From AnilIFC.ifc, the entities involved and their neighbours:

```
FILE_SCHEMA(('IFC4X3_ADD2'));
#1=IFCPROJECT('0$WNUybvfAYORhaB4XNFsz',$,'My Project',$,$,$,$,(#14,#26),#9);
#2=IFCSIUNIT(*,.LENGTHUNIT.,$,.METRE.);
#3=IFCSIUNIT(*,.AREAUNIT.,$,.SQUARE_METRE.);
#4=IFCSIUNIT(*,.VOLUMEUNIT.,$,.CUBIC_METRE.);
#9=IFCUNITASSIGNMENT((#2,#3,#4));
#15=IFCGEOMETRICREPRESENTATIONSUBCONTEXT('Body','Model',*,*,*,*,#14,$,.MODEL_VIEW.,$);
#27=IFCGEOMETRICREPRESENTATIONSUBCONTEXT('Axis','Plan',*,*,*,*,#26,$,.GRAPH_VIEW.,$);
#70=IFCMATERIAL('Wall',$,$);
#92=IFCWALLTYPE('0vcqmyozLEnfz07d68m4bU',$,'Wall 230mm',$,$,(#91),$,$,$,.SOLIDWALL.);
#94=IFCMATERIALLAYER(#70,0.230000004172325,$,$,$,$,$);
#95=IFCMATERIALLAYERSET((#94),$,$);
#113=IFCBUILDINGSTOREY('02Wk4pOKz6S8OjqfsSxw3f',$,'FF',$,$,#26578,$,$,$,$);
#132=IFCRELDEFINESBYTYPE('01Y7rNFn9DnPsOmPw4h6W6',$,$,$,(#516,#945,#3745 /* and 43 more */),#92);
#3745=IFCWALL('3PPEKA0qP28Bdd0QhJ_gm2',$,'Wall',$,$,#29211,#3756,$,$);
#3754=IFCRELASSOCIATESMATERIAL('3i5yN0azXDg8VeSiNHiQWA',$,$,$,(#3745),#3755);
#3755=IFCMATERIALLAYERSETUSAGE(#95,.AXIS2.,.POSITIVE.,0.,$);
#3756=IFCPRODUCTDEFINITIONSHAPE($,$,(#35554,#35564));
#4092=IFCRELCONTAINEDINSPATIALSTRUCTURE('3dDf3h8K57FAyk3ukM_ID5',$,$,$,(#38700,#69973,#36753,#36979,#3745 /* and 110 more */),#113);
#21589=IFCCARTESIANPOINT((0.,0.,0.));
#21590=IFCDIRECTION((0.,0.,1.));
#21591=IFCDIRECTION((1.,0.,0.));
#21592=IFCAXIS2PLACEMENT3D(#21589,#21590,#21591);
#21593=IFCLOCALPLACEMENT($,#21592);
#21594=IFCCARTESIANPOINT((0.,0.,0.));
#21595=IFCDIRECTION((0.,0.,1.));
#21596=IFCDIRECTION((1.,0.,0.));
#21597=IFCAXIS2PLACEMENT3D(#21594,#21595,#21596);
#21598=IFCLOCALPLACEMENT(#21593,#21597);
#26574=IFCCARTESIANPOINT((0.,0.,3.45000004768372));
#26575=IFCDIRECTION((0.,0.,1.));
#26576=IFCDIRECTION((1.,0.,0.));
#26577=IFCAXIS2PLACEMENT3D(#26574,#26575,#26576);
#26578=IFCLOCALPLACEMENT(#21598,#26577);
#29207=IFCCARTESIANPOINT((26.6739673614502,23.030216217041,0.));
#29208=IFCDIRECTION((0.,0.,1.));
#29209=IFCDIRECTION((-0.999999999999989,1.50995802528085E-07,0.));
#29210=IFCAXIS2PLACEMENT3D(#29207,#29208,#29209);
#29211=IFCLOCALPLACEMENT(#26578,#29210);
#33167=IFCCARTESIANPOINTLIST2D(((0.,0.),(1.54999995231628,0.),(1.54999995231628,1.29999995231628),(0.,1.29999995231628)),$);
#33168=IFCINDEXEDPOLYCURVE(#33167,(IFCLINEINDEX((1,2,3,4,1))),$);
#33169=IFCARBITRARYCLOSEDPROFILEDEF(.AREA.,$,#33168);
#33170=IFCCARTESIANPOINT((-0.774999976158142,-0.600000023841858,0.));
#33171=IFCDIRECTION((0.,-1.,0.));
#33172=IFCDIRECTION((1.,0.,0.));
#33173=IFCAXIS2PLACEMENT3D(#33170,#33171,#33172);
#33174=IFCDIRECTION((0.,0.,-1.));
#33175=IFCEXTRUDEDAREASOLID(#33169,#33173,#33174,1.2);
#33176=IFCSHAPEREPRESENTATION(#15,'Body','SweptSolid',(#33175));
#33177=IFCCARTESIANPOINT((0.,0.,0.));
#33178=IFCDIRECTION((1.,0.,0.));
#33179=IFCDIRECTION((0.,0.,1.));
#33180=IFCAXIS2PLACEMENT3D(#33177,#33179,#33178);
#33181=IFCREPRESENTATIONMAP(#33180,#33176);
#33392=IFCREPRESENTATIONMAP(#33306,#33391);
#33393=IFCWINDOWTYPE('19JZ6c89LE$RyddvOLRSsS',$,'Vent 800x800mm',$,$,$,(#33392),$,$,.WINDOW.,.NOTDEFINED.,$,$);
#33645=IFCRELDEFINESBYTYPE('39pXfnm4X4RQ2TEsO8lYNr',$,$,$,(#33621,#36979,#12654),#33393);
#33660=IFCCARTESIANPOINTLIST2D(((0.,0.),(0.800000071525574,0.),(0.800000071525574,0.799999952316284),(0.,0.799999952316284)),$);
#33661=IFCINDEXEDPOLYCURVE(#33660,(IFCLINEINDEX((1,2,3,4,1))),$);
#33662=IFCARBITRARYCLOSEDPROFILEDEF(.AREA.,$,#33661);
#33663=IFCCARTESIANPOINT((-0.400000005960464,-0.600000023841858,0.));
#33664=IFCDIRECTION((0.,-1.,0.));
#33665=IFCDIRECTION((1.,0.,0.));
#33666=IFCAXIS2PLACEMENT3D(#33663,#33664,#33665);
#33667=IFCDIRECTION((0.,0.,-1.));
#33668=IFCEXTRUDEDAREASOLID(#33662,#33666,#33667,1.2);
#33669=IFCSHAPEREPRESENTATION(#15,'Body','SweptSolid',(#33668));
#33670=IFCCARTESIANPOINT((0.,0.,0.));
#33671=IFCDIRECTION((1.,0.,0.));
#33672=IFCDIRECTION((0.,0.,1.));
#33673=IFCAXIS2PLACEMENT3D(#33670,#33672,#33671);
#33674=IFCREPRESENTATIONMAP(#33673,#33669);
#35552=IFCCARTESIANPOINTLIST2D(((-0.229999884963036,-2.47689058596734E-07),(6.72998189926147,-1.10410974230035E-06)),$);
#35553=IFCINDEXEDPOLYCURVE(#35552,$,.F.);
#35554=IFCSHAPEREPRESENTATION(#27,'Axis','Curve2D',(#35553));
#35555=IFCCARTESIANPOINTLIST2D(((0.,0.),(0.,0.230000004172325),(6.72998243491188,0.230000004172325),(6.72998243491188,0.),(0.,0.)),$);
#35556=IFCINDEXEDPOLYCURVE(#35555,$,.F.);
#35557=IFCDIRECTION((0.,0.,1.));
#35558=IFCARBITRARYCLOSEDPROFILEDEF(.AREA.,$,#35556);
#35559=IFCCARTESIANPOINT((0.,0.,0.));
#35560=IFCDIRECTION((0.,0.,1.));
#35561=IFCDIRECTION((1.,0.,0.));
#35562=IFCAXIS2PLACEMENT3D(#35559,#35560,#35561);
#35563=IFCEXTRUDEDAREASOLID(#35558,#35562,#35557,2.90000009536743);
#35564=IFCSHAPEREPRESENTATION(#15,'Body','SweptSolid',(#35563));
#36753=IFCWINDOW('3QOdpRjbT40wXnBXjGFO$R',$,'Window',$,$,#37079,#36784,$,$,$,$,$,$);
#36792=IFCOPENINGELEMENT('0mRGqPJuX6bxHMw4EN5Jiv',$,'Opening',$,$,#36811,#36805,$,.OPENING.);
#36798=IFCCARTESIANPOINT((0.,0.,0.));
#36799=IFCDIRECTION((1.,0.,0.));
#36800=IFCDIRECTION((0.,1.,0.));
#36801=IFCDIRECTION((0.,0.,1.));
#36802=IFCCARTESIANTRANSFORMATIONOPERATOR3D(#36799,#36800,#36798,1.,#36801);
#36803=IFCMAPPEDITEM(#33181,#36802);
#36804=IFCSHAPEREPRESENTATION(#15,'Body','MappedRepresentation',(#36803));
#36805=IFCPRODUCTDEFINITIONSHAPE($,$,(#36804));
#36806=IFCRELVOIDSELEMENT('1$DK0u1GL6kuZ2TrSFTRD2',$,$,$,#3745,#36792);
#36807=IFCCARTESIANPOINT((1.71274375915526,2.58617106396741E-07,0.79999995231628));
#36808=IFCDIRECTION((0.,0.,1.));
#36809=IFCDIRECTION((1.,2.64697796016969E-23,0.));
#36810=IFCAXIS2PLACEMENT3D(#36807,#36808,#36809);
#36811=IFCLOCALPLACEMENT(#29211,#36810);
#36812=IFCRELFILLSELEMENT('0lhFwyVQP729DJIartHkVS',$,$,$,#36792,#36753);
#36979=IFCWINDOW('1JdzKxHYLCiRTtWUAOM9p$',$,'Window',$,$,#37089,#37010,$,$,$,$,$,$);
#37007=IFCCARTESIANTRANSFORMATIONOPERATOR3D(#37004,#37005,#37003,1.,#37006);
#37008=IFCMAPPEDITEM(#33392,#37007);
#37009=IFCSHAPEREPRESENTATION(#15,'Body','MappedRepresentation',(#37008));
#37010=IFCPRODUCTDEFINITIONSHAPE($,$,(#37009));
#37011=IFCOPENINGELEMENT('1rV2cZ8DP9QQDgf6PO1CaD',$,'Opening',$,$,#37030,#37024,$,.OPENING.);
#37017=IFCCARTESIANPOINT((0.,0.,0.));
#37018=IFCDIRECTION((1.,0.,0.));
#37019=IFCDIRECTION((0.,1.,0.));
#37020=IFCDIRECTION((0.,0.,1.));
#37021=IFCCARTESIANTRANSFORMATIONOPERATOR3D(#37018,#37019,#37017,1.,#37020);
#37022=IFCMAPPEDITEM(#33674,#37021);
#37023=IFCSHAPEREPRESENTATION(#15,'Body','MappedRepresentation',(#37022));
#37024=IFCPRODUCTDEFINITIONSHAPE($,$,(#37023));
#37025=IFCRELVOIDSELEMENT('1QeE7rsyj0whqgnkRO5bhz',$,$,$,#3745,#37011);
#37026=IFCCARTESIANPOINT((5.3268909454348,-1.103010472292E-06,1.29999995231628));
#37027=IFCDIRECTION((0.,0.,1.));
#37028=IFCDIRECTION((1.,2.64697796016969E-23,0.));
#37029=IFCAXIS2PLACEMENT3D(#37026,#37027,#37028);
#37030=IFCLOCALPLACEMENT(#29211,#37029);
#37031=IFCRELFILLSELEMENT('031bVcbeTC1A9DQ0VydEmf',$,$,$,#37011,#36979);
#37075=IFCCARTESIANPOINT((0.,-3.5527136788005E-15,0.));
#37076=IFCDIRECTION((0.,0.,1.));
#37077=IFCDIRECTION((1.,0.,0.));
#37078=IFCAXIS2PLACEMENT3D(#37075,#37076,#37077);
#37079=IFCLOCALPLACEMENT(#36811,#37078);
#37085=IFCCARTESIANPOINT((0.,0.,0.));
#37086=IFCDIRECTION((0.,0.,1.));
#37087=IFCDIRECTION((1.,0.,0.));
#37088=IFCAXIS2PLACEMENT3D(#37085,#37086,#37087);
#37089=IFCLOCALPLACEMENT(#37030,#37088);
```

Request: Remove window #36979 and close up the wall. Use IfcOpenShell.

```python
import ifcopenshell
import ifcopenshell.api.feature
import ifcopenshell.api.root
import ifcopenshell.geom
import ifcopenshell.util.shape

model = ifcopenshell.open("AnilIFC.ifc")
settings = ifcopenshell.geom.settings()


def volume(element):
    """Net volume in cubic metres, openings subtracted."""
    shape = ifcopenshell.geom.create_shape(settings, element)
    return ifcopenshell.util.shape.get_volume(shape.geometry)


window = model.by_guid("1JdzKxHYLCiRTtWUAOM9p$")
opening = window.FillsVoids[0].RelatingOpeningElement
wall = opening.VoidsElements[0].RelatingBuildingElement
before = volume(wall)

ifcopenshell.api.root.remove_product(model, product=window)
ifcopenshell.api.feature.remove_feature(model, feature=opening)

after = volume(wall)

print(f"wall volume {before:.3f} -> {after:.3f} m3")

model.write("AnilIFC_edited.ifc")
```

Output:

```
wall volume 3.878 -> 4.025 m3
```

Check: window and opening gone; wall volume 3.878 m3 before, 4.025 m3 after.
